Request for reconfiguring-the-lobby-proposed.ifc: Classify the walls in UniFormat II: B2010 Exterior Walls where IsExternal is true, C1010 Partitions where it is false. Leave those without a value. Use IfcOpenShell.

First a look at what the model holds.

```python
import ifcopenshell
import ifcopenshell.util.element

model = ifcopenshell.open("reconfiguring-the-lobby-proposed.ifc")
print(model.schema)
print("classifications:", [c.Name for c in model.by_type("IfcClassification")])
values = [ifcopenshell.util.element.get_pset(e, "Pset_WallCommon", "IsExternal") for e in model.by_type("IfcWall")]
for value in (True, False, None):
    print("IsExternal", value, values.count(value))
```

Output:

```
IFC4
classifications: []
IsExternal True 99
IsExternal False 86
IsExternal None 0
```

```python
import ifcopenshell
import ifcopenshell.api.classification
import ifcopenshell.util.element

model = ifcopenshell.open("reconfiguring-the-lobby-proposed.ifc")

system = ifcopenshell.api.classification.add_classification(model, classification="UniFormat II")

walls = model.by_type("IfcWall")
external = {e: ifcopenshell.util.element.get_pset(e, "Pset_WallCommon", "IsExternal") for e in walls}
for flag, code, name in ((True, "B2010", "Exterior Walls"), (False, "C1010", "Partitions")):
    products = [e for e in walls if external[e] is flag]
    ifcopenshell.api.classification.add_reference(
        model, products=products, classification=system, identification=code, name=name
    )
    print(code, len(products))

model.write("reconfiguring-the-lobby-proposed_rev.ifc")
```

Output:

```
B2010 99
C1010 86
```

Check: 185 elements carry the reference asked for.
